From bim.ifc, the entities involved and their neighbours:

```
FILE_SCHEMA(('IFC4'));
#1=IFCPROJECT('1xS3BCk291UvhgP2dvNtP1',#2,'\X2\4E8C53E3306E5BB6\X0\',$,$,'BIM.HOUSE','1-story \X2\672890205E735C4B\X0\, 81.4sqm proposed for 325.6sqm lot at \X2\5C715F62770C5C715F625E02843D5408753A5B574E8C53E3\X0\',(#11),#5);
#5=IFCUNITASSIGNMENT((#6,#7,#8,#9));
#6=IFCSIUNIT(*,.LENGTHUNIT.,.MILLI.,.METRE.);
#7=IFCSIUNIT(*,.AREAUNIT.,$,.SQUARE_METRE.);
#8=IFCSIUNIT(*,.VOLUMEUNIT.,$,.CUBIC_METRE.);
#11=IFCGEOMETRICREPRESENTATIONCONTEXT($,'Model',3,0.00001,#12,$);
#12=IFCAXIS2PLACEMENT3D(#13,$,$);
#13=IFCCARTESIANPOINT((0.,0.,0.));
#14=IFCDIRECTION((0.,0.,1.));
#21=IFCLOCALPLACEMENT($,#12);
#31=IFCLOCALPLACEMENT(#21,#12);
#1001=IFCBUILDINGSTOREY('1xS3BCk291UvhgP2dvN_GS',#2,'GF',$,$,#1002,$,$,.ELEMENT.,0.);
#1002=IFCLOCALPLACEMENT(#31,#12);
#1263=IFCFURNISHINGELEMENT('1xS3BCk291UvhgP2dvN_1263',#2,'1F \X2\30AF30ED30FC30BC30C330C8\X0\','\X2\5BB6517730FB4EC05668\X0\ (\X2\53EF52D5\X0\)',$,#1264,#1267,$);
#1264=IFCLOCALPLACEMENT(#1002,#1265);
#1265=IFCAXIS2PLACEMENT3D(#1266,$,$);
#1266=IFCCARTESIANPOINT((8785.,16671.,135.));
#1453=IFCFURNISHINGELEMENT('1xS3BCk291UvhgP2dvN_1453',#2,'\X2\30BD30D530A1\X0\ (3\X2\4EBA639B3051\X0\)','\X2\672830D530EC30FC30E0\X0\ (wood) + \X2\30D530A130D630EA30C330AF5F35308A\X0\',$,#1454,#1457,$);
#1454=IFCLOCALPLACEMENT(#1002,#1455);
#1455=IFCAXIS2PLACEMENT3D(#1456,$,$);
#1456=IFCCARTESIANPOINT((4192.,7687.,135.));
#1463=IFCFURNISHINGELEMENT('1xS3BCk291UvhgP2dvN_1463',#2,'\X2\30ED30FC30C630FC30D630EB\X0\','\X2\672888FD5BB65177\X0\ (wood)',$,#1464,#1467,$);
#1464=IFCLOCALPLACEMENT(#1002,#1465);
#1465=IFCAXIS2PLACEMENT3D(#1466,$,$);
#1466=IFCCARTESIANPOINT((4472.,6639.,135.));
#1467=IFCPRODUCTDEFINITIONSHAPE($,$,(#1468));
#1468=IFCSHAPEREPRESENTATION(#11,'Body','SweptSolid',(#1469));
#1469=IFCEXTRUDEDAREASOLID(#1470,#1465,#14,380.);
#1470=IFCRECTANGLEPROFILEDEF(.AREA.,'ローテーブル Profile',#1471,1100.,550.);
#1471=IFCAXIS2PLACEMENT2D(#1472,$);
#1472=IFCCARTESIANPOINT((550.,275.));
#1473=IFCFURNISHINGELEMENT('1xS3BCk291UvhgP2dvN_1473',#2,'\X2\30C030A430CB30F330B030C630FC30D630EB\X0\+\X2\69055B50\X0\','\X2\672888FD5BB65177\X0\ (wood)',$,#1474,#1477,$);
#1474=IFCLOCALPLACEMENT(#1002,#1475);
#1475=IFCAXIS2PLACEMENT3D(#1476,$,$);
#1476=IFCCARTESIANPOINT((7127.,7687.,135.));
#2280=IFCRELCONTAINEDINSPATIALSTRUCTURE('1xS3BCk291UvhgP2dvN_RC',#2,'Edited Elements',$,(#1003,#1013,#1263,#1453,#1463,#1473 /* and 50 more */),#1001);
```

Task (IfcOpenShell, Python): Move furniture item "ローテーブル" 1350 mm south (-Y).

```python
import ifcopenshell
import ifcopenshell.api.geometry
import ifcopenshell.util.placement
import ifcopenshell.util.unit

model = ifcopenshell.open("bim.ifc")
unit_scale = ifcopenshell.util.unit.calculate_unit_scale(model)

item = model.by_id(1463)
matrix = ifcopenshell.util.placement.get_local_placement(item.ObjectPlacement)
matrix[1, 3] -= 1.35 / unit_scale
ifcopenshell.api.geometry.edit_object_placement(model, product=item, matrix=matrix, is_si=False)

print(ifcopenshell.util.placement.get_local_placement(item.ObjectPlacement).round(3) + 0.0)

model.write("bim_v2.ifc")
```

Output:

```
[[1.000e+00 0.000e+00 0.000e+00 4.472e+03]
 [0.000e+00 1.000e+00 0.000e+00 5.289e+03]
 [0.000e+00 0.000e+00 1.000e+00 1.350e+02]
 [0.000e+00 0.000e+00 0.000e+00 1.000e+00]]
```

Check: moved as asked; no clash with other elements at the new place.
